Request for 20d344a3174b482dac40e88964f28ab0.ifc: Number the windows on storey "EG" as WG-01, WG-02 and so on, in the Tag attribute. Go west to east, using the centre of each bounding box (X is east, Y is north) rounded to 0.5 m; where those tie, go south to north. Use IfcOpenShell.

First a look at what the model holds.

```python
import ifcopenshell
import ifcopenshell.util.element
import ifcopenshell.util.placement

model = ifcopenshell.open("20d344a3174b482dac40e88964f28ab0.ifc")
print(model.schema)
storey = next(s for s in model.by_type("IfcBuildingStorey") if s.Name == "EG")
windows = [e for e in ifcopenshell.util.element.get_decomposition(storey) if e.is_a("IfcWindow")]
for e in sorted(windows, key=lambda e: e.id()):
    origin = ifcopenshell.util.placement.get_local_placement(e.ObjectPlacement)[:3, 3]
    print(e.id(), e.Tag, e.Name, origin.round(2) + 0.0, sep=" | ")
```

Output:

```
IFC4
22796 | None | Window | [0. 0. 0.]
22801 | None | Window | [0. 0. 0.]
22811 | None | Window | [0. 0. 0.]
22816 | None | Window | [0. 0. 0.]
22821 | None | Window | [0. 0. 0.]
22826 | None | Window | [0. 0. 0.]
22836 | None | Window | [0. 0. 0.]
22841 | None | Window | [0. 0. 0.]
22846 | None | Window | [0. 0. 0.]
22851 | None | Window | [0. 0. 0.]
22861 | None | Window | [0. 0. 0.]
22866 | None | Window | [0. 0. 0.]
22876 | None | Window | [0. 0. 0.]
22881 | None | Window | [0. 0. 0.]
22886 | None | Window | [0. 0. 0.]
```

```python
import ifcopenshell
import ifcopenshell.geom
import ifcopenshell.util.element
import ifcopenshell.util.shape

model = ifcopenshell.open("20d344a3174b482dac40e88964f28ab0.ifc")
settings = ifcopenshell.geom.settings()
settings.set("use-world-coords", True)


def centre(element):
    shape = ifcopenshell.geom.create_shape(settings, element)
    return ifcopenshell.util.shape.get_bbox_centroid(shape.geometry)


storey = next(s for s in model.by_type("IfcBuildingStorey") if s.Name == "EG")
windows = [e for e in ifcopenshell.util.element.get_decomposition(storey) if e.is_a("IfcWindow")]

# Insertion points can sit at a corner or the storey origin, so sort by the geometry (in metres).
centres = {e: centre(e) for e in windows}
windows.sort(key=lambda e: (round(centres[e][0] / 0.5), centres[e][1]))

for i, e in enumerate(windows, start=1):
    number = f"WG-{i:02d}"
    e.Tag = number
    print(e.id(), number)

model.write("20d344a3174b482dac40e88964f28ab0-out.ifc")
```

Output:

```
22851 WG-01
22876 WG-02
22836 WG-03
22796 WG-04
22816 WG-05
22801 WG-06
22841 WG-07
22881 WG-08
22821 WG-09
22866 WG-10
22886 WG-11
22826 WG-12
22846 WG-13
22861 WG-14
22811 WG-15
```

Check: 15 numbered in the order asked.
